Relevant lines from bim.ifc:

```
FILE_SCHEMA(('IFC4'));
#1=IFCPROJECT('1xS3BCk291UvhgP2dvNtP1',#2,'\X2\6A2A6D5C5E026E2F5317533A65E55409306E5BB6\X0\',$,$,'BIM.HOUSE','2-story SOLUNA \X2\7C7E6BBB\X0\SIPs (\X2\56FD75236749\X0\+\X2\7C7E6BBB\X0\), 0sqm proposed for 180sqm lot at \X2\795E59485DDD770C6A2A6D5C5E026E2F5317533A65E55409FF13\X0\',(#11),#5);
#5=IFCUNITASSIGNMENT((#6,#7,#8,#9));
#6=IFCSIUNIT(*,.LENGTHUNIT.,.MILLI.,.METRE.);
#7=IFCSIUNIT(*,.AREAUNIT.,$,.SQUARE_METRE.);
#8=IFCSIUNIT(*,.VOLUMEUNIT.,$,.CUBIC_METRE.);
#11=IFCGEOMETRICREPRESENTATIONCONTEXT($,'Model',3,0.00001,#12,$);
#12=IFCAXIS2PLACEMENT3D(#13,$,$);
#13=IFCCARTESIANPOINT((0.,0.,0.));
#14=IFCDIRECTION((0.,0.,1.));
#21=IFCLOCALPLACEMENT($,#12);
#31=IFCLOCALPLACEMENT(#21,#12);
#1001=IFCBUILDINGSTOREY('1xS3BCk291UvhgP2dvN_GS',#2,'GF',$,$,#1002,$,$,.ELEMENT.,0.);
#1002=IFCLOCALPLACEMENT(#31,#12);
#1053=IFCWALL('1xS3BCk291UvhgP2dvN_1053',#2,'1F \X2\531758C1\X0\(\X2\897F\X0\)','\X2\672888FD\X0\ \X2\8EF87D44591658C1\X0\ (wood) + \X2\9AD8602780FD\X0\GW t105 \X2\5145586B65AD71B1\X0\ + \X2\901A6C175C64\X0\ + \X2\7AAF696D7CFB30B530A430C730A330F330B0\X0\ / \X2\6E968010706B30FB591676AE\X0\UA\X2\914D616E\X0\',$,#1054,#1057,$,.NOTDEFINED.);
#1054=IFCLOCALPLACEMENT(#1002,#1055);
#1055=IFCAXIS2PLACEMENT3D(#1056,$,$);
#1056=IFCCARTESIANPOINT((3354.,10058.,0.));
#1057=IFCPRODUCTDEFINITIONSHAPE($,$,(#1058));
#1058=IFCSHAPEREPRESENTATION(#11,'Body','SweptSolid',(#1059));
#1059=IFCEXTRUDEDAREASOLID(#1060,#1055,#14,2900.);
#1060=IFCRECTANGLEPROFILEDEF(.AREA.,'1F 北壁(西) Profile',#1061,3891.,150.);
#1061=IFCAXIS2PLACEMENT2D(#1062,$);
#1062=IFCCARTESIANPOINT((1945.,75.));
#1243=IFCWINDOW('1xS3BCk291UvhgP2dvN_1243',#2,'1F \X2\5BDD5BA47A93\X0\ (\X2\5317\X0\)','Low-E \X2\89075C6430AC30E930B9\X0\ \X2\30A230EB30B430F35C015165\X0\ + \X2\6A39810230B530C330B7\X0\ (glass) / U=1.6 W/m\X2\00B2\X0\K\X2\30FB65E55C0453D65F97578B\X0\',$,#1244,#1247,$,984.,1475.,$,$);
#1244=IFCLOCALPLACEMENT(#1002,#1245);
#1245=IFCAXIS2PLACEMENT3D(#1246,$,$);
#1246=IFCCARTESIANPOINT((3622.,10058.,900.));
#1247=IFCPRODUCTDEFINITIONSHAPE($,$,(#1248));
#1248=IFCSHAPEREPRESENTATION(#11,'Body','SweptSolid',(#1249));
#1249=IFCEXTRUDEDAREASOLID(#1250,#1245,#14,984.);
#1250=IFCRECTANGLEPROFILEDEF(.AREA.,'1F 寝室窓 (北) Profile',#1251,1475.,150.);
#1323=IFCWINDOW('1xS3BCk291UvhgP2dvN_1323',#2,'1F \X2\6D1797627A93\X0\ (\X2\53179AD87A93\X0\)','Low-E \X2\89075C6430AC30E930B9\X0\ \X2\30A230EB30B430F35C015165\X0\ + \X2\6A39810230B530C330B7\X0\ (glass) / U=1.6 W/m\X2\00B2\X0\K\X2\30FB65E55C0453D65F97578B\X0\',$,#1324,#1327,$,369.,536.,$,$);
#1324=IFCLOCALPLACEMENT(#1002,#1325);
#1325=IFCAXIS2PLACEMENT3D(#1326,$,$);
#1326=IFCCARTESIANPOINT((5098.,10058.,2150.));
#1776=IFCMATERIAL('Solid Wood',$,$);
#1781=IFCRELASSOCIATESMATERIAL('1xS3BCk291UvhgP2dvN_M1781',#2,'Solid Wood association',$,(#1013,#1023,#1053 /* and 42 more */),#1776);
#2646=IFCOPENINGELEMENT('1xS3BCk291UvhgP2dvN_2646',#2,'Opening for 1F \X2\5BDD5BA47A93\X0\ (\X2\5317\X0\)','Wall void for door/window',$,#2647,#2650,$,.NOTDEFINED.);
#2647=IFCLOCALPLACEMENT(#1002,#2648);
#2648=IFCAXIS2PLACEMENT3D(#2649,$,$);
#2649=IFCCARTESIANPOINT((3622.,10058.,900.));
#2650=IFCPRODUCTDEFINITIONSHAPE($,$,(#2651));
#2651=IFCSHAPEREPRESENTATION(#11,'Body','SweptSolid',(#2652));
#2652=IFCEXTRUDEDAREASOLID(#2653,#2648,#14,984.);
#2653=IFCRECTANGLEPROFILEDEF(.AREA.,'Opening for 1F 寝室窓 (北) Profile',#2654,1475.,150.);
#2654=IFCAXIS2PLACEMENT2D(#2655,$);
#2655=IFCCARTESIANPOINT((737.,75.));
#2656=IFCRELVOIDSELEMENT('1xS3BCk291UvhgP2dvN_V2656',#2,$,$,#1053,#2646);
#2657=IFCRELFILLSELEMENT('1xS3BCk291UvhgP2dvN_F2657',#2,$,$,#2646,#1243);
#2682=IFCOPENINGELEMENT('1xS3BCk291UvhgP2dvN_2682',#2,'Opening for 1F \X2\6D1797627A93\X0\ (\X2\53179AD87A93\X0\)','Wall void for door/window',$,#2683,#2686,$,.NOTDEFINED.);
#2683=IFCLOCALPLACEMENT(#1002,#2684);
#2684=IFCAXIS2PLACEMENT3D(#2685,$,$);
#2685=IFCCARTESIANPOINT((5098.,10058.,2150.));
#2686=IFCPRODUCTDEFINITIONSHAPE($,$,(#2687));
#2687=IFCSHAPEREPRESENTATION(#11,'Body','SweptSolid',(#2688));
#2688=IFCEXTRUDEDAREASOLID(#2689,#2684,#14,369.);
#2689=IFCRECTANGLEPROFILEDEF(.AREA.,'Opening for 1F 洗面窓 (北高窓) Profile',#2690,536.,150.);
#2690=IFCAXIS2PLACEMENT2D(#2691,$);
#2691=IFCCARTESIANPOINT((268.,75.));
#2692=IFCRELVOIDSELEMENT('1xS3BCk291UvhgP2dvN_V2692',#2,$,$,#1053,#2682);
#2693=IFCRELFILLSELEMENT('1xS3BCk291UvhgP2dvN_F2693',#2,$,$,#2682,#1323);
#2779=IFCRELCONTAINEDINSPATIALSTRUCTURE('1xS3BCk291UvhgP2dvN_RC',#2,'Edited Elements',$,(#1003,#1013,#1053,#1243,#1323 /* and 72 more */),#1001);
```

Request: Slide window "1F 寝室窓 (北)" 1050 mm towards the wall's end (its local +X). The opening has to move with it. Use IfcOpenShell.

```python
import ifcopenshell
import ifcopenshell.api.geometry
import ifcopenshell.util.placement

model = ifcopenshell.open("bim.ifc")

window = model.by_guid("1xS3BCk291UvhgP2dvN_1243")
opening = window.FillsVoids[0].RelatingOpeningElement
wall = opening.VoidsElements[0].RelatingBuildingElement

wall_matrix = ifcopenshell.util.placement.get_local_placement(wall.ObjectPlacement)
shift = wall_matrix[:3, 0] * 1050.0
before = ifcopenshell.util.placement.get_local_placement(window.ObjectPlacement)[:3, 3].copy()

# The window is not placed relative to its opening, so move both.
for product in (opening, window):
    matrix = ifcopenshell.util.placement.get_local_placement(product.ObjectPlacement)
    matrix[:3, 3] += shift
    ifcopenshell.api.geometry.edit_object_placement(model, product=product, matrix=matrix, is_si=False)

after = ifcopenshell.util.placement.get_local_placement(window.ObjectPlacement)[:3, 3]
print("window moved by", (after - before).round(3) + 0.0)

model.write("bim_v2.ifc")
```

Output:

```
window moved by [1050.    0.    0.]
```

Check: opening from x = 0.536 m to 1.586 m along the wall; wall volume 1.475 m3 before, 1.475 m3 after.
